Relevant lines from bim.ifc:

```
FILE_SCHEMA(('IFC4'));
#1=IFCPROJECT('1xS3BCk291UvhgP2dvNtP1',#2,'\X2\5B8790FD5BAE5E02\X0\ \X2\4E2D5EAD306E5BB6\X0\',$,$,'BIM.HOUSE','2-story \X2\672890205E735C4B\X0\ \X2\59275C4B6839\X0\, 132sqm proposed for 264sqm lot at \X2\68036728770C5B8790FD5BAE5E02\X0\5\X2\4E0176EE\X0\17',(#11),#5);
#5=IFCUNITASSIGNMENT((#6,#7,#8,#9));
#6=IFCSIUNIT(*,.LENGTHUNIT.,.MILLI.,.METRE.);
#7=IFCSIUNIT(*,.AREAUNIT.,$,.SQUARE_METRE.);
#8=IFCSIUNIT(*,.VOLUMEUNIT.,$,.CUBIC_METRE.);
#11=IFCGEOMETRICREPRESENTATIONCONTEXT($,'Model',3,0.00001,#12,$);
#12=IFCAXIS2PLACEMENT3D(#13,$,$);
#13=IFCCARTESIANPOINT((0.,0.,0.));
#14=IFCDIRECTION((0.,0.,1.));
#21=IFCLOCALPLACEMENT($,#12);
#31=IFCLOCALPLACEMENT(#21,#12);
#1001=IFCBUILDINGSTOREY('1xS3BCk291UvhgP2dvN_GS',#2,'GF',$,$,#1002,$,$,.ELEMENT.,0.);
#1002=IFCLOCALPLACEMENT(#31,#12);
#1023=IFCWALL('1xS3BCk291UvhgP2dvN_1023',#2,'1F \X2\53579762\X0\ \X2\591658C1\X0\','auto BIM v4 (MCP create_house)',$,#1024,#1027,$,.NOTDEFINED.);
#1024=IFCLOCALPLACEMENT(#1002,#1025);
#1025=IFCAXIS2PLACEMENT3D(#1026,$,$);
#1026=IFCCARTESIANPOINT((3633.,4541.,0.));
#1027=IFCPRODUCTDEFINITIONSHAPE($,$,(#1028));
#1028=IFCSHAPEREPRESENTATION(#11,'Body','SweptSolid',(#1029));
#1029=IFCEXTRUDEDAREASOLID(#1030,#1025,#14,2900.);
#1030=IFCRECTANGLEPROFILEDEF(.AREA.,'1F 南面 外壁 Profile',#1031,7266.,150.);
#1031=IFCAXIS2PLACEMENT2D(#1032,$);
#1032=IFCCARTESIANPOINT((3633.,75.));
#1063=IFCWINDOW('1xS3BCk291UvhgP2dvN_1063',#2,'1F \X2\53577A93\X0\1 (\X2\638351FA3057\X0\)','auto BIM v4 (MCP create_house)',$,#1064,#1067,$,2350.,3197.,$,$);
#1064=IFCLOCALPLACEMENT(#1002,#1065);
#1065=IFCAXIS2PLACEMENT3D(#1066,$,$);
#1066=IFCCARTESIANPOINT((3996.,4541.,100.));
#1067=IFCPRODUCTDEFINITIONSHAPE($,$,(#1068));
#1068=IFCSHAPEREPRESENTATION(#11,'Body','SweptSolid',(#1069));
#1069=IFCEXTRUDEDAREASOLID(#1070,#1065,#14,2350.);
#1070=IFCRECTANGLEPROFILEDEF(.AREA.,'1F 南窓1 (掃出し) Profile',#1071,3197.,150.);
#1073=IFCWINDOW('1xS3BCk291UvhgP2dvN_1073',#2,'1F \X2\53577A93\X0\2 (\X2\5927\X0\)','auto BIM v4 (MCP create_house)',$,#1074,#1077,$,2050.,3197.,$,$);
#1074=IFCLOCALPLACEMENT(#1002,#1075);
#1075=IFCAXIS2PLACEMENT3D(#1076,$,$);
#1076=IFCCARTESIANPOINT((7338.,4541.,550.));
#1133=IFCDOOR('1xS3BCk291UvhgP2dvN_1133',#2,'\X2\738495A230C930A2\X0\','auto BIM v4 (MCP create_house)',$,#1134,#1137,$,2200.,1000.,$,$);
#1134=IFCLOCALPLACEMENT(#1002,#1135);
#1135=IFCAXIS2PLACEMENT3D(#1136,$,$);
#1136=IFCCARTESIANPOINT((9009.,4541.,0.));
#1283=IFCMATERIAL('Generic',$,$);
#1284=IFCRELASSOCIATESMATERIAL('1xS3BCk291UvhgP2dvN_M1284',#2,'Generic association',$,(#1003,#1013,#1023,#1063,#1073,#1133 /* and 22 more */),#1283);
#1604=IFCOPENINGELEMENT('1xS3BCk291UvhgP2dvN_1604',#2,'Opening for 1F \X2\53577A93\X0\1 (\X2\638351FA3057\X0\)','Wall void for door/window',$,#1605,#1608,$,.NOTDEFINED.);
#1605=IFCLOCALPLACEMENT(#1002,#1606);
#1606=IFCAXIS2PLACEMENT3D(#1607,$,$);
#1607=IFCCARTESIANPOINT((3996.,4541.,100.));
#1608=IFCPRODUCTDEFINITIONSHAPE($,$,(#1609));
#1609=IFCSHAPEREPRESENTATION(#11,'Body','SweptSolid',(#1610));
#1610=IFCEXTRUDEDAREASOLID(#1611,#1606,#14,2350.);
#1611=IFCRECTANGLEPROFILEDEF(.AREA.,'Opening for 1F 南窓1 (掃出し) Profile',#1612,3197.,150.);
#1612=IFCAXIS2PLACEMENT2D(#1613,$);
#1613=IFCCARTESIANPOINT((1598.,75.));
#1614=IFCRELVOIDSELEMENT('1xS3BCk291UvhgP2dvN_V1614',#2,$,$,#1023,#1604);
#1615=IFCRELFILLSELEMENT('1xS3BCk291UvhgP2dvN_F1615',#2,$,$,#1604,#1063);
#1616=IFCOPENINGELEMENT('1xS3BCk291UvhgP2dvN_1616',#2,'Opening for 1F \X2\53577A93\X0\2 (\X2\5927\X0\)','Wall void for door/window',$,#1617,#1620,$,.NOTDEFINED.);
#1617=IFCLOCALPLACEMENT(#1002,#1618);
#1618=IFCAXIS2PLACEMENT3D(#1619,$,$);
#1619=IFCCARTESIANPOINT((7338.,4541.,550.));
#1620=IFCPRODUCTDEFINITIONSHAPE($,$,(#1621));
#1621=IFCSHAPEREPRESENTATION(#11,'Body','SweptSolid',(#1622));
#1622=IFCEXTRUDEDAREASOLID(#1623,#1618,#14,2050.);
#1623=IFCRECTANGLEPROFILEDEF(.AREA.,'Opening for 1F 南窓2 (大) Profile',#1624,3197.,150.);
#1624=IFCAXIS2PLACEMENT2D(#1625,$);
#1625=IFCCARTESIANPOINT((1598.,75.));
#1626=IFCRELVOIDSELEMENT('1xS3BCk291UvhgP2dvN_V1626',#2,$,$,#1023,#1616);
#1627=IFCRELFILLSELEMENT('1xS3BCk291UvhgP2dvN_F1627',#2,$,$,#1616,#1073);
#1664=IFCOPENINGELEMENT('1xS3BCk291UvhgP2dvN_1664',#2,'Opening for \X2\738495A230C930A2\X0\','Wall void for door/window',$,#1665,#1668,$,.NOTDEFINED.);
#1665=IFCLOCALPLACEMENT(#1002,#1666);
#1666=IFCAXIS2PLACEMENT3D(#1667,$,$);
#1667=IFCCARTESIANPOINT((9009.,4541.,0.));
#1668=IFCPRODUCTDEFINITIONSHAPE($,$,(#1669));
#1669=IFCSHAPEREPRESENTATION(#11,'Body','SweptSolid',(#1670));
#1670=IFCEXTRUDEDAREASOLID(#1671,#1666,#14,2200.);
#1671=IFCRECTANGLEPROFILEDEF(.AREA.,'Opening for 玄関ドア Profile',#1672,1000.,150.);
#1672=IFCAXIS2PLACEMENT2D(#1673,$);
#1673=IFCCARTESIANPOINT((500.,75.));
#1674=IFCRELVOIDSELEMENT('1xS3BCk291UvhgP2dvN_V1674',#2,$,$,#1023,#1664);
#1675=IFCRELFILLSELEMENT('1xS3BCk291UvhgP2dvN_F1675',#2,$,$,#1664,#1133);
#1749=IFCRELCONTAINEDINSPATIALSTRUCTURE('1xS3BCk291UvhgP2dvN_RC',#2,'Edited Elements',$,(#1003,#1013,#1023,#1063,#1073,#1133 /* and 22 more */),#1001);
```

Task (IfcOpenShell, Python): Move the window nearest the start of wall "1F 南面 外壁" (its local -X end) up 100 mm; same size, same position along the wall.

```python
import numpy as np
import ifcopenshell
import ifcopenshell.api.geometry
import ifcopenshell.util.placement
import ifcopenshell.util.unit

model = ifcopenshell.open("bim.ifc")
unit_scale = ifcopenshell.util.unit.calculate_unit_scale(model)

window = model.by_guid("1xS3BCk291UvhgP2dvN_1063")
opening = window.FillsVoids[0].RelatingOpeningElement
dz = 0.1 / unit_scale

shift = np.array([0.0, 0.0, dz])
# The window is not placed relative to its opening, so move both.
for product in (opening, window):
    matrix = ifcopenshell.util.placement.get_local_placement(product.ObjectPlacement)
    matrix[:3, 3] += shift
    ifcopenshell.api.geometry.edit_object_placement(model, product=product, matrix=matrix, is_si=False)

print(f"moved by {dz * unit_scale:+.3f} m")

model.write("bim_edited.ifc")
```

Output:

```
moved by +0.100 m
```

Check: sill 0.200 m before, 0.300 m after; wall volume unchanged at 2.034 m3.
